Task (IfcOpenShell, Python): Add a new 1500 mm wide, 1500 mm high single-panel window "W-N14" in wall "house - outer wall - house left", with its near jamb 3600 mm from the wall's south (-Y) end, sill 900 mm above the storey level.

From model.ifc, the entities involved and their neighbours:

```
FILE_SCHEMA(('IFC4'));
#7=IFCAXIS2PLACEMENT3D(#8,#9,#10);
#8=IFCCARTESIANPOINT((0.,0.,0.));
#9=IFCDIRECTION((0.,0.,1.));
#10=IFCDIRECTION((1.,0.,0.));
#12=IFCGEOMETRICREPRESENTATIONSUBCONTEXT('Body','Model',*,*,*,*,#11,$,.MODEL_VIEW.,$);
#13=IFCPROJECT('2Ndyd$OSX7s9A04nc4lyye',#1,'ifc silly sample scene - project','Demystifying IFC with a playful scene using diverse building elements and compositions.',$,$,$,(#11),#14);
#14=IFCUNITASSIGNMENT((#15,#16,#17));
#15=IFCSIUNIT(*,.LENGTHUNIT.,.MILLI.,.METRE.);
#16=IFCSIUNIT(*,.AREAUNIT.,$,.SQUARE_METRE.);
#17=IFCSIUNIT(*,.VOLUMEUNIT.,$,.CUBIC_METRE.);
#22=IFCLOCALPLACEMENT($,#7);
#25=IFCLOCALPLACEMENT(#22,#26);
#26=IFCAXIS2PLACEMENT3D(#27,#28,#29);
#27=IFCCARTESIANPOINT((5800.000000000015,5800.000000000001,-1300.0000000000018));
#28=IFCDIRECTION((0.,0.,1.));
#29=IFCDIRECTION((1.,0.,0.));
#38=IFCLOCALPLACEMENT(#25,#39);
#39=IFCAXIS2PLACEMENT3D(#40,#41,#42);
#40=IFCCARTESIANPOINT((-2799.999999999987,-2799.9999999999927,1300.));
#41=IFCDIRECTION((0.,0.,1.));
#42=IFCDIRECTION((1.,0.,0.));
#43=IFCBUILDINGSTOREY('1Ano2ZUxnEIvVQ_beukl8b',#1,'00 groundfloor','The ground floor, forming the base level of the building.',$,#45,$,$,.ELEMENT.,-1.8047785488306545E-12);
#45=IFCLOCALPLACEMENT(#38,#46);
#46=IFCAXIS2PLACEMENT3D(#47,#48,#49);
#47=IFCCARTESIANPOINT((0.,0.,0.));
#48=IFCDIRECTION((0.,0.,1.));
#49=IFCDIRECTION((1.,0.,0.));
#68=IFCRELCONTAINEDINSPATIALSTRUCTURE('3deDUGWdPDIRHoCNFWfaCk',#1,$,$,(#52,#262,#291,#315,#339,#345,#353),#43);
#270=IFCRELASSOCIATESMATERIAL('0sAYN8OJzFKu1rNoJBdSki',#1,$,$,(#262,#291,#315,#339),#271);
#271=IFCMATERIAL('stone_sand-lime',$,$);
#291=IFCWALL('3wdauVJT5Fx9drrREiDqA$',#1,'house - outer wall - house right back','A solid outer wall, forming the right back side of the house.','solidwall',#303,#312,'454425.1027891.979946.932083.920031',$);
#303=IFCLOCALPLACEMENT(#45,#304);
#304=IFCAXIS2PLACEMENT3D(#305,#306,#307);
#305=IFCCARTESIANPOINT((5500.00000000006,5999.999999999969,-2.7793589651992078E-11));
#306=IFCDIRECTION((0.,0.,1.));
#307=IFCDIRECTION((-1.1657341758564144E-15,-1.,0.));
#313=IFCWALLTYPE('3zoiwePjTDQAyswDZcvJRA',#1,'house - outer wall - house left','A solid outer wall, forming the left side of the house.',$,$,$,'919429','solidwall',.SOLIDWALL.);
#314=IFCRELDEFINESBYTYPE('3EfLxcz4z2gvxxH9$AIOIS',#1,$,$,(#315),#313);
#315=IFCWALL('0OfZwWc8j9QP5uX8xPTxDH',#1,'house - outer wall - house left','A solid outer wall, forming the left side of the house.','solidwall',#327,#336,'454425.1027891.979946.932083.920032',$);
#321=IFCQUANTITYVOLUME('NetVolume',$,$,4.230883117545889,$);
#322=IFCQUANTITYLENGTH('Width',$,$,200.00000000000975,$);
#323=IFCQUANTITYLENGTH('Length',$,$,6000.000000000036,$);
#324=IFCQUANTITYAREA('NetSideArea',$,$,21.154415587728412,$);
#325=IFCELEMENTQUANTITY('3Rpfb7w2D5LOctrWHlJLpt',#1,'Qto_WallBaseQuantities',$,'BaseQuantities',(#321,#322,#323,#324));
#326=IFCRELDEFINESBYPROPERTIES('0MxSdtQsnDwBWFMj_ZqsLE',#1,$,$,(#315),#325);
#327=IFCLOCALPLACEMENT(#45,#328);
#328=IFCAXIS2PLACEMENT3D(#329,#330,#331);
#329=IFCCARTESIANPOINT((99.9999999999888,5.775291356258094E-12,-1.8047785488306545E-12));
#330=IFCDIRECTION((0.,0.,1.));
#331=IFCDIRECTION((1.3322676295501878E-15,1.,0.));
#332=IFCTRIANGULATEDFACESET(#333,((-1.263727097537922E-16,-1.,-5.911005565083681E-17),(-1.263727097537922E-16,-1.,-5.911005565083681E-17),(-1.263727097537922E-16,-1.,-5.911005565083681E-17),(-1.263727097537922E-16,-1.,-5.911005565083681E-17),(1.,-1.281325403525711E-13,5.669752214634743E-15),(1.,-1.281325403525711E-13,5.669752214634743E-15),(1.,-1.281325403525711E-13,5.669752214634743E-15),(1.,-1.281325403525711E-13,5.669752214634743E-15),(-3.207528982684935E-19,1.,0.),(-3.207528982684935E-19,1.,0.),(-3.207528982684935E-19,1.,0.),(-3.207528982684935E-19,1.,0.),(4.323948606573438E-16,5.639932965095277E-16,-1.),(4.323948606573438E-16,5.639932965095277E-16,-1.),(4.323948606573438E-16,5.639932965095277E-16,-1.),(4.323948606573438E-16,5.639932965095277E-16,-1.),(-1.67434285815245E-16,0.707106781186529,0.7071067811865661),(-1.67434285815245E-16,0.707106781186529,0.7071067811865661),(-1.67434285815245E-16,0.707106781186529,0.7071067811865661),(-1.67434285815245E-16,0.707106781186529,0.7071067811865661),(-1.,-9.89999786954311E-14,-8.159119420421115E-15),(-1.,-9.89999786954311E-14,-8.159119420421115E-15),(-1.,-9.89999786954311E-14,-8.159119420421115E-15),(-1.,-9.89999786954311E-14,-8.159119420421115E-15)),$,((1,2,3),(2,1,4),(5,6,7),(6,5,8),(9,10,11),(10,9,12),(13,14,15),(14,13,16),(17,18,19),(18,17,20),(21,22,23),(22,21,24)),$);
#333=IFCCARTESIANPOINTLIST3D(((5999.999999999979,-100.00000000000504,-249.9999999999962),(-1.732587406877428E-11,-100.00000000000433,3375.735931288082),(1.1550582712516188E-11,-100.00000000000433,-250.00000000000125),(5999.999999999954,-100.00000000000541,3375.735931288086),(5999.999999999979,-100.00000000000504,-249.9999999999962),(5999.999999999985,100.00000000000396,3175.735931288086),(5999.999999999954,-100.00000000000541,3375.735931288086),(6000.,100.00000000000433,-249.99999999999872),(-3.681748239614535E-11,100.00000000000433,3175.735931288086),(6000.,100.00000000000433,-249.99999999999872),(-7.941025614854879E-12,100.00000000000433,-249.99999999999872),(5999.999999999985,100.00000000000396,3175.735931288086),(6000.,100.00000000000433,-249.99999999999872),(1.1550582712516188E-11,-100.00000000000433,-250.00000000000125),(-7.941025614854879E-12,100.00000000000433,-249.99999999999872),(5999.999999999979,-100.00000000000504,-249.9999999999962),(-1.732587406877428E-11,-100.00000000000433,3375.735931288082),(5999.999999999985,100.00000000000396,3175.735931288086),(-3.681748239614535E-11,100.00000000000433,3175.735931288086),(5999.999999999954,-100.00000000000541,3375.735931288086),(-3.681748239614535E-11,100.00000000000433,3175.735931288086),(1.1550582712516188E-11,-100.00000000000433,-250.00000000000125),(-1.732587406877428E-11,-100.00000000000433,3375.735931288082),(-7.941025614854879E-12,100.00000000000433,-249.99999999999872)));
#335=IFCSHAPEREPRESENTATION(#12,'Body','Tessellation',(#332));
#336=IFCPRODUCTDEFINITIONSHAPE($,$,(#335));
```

```python
import numpy as np
import ifcopenshell
import ifcopenshell.api.feature
import ifcopenshell.api.geometry
import ifcopenshell.api.pset
import ifcopenshell.api.root
import ifcopenshell.api.spatial
import ifcopenshell.geom
import ifcopenshell.util.element
import ifcopenshell.util.placement
import ifcopenshell.util.representation
import ifcopenshell.util.shape
import ifcopenshell.util.unit

model = ifcopenshell.open("model.ifc")
unit_scale = ifcopenshell.util.unit.calculate_unit_scale(model)
area_scale = ifcopenshell.util.unit.calculate_unit_scale(model, "AREAUNIT")
volume_scale = ifcopenshell.util.unit.calculate_unit_scale(model, "VOLUMEUNIT")
settings = ifcopenshell.geom.settings()


def volume(element):
    """Net volume in cubic metres, openings subtracted."""
    shape = ifcopenshell.geom.create_shape(settings, element)
    return ifcopenshell.util.shape.get_volume(shape.geometry)


wall = model.by_id(315)
storey = ifcopenshell.util.element.get_container(wall, ifc_class="IfcBuildingStorey")
context = ifcopenshell.util.representation.get_context(model, "Model", "Body", "MODEL_VIEW")
before = volume(wall)

width, height, from_end, sill = 1.5, 1.5, 3.6, 0.9  # metres

# The wall runs along its own X axis, and the end named is its -X end.
wall_shape = ifcopenshell.geom.create_shape(settings, wall)
x, y, z = ifcopenshell.util.shape.get_vertices(wall_shape.geometry).T
start = x.min() + from_end
face, thickness = float(y.min()), float(y.max() - y.min())
wall_matrix = ifcopenshell.util.placement.get_local_placement(wall.ObjectPlacement)
level = ifcopenshell.util.placement.get_local_placement(storey.ObjectPlacement)[2, 3]


def in_wall(x, y):
    """Placement at x, y metres in the wall's axes, at sill height."""
    matrix = wall_matrix.copy()
    matrix[:, 3] = wall_matrix @ np.array([x / unit_scale, y / unit_scale, 0.0, 1.0])
    matrix[2, 3] = level + sill / unit_scale
    return matrix


# Opening: a box that overshoots both wall faces by 50 mm.
opening = ifcopenshell.api.root.create_entity(model, ifc_class="IfcOpeningElement", predefined_type="OPENING")
box = ifcopenshell.api.geometry.add_wall_representation(
    model, context=context, length=width, height=height, thickness=thickness + 0.1
)
ifcopenshell.api.geometry.assign_representation(model, product=opening, representation=box)
ifcopenshell.api.geometry.edit_object_placement(model, product=opening, matrix=in_wall(start, face - 0.05), is_si=False)
ifcopenshell.api.feature.add_feature(model, feature=opening, element=wall)

window = ifcopenshell.api.root.create_entity(model, ifc_class="IfcWindow", name="W-N14", predefined_type="WINDOW")
window.OverallWidth, window.OverallHeight = width / unit_scale, height / unit_scale
window.PartitioningType = "SINGLE_PANEL"
body = ifcopenshell.api.geometry.add_window_representation(
    model,
    context=context,
    overall_width=window.OverallWidth,
    overall_height=window.OverallHeight,
    partition_type="SINGLE_PANEL",
)
ifcopenshell.api.geometry.assign_representation(model, product=window, representation=body)
ifcopenshell.api.spatial.assign_container(model, products=[window], relating_structure=storey)
ifcopenshell.api.feature.add_filling(model, opening=opening, element=window)

# Centre the window in the wall's thickness.
ifcopenshell.api.geometry.edit_object_placement(model, product=window, matrix=in_wall(start, face), is_si=False)
window_shape = ifcopenshell.geom.create_shape(settings, window)
depth = ifcopenshell.util.shape.get_vertices(window_shape.geometry)[:, 1]
offset = face + thickness / 2 - (depth.min() + depth.max()) / 2
ifcopenshell.api.geometry.edit_object_placement(model, product=window, matrix=in_wall(start, offset), is_si=False)

after = volume(wall)

# Update the wall's stored quantities.
qto = model.by_id(ifcopenshell.util.element.get_pset(wall, "Qto_WallBaseQuantities", should_inherit=False)["id"])
ifcopenshell.api.pset.edit_qto(model, qto=qto, properties={
    "NetVolume": after / volume_scale,
    "NetSideArea": after / thickness / area_scale,
})

print(f"wall volume {before:.3f} -> {after:.3f} m3")

model.write("model-out.ifc")
```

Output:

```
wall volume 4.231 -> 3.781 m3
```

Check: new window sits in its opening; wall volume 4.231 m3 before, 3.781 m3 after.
